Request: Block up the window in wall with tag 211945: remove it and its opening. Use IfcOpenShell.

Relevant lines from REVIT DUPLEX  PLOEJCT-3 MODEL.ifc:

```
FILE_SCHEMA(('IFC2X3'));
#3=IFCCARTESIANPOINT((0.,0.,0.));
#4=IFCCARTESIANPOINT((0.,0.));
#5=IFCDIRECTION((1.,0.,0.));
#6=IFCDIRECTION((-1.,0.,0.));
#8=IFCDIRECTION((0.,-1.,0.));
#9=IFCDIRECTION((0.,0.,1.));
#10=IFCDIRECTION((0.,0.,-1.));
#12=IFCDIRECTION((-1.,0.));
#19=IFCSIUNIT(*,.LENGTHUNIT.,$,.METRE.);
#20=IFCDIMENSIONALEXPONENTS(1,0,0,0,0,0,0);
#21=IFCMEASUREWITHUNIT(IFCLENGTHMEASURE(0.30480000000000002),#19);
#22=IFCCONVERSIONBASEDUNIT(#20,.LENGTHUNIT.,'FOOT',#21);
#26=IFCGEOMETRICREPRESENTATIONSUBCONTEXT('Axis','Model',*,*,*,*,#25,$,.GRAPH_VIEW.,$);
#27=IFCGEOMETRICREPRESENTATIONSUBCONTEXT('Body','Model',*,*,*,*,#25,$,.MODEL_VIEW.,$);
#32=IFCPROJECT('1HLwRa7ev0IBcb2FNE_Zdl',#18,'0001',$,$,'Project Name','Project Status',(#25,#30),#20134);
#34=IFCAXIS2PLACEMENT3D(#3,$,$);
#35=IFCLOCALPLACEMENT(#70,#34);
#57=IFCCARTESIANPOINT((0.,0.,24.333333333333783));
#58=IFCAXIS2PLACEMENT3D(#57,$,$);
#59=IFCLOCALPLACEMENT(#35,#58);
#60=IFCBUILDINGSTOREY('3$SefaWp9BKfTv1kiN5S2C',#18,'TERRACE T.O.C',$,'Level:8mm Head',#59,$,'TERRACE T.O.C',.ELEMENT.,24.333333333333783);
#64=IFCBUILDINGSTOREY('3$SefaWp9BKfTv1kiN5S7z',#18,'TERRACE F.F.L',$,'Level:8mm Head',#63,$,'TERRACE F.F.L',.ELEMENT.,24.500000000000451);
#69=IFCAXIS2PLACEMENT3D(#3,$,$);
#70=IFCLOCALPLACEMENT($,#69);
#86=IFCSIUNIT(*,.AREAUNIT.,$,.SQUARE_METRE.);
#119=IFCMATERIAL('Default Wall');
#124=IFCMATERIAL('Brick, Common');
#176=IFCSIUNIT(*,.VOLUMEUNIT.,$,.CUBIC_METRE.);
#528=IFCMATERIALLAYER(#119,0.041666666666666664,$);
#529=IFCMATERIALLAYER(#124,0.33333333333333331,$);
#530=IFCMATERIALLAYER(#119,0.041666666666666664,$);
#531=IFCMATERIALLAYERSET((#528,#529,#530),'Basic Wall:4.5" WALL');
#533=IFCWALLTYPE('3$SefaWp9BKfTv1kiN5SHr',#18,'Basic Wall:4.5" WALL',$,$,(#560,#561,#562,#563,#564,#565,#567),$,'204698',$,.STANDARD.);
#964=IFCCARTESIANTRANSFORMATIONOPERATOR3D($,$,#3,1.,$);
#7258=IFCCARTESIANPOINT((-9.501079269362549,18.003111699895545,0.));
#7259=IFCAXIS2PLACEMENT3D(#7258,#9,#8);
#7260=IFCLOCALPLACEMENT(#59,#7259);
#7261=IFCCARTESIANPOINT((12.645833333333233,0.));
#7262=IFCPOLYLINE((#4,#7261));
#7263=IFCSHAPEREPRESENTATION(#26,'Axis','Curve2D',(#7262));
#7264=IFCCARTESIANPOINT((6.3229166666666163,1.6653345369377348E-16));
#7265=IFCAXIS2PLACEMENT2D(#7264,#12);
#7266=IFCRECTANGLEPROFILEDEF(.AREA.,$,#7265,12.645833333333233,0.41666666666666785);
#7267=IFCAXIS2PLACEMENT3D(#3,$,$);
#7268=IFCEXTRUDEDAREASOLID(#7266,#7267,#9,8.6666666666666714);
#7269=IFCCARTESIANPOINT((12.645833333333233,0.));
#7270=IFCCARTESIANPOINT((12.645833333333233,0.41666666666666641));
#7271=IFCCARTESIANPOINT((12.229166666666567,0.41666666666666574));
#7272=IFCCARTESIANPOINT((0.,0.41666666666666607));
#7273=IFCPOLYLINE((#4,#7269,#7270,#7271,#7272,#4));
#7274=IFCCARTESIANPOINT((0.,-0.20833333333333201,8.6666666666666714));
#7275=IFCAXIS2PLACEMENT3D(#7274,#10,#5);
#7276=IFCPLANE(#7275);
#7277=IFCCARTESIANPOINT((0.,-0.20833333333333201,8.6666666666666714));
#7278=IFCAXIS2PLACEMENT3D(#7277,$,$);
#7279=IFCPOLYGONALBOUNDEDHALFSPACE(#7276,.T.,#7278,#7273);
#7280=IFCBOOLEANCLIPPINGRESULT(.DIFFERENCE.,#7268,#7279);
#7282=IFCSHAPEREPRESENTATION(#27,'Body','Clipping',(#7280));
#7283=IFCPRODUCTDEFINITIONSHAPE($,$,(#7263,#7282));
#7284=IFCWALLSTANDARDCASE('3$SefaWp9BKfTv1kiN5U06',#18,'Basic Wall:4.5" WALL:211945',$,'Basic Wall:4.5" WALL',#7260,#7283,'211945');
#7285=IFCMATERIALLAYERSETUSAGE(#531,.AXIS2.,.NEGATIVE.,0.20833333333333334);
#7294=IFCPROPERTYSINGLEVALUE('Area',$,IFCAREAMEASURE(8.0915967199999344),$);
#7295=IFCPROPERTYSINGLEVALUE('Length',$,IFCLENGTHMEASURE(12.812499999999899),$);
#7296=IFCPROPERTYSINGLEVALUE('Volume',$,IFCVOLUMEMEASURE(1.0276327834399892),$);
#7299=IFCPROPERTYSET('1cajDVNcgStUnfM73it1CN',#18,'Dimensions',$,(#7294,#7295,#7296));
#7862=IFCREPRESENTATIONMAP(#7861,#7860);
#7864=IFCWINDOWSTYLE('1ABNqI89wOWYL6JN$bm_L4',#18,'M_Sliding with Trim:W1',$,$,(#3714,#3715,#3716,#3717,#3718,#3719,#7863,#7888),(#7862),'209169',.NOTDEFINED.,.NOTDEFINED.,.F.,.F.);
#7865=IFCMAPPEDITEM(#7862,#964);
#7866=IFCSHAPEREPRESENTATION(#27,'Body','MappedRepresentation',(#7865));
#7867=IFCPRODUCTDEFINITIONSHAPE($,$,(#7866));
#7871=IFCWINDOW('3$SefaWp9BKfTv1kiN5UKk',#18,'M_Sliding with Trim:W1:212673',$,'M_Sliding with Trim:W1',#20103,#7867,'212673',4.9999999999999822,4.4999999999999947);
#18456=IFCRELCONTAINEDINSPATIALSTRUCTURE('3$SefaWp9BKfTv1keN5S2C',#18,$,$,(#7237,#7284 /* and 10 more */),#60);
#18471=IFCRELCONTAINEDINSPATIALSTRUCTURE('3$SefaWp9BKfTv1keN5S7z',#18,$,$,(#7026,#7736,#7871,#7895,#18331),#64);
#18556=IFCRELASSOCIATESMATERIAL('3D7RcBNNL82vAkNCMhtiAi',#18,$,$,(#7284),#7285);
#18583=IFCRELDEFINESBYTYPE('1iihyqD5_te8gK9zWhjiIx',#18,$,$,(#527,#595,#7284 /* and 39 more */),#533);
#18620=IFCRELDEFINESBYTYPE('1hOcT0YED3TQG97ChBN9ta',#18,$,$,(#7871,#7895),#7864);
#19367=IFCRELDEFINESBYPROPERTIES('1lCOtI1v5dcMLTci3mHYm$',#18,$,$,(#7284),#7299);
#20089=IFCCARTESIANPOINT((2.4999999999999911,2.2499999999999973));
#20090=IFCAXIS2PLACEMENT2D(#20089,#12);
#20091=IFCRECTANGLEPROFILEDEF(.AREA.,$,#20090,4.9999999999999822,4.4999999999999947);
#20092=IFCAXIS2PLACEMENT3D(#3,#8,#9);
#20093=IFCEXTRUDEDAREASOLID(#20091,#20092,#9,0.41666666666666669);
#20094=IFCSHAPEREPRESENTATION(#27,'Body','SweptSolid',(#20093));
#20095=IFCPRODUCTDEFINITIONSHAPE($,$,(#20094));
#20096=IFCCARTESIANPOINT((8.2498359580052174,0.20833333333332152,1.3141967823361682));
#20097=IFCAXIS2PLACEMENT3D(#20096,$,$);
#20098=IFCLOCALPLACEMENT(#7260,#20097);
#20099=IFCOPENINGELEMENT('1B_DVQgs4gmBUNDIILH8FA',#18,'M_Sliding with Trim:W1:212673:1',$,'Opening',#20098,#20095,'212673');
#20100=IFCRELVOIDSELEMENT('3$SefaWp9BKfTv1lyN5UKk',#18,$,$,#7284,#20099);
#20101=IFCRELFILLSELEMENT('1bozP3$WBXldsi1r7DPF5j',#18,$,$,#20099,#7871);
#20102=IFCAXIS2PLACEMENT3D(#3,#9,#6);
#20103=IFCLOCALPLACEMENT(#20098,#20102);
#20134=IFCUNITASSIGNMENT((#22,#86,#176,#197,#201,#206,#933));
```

```python
import ifcopenshell
import ifcopenshell.api.feature
import ifcopenshell.api.pset
import ifcopenshell.api.root
import ifcopenshell.geom
import ifcopenshell.util.element
import ifcopenshell.util.shape
import ifcopenshell.util.unit

model = ifcopenshell.open("REVIT DUPLEX  PLOEJCT-3 MODEL.ifc")
area_scale = ifcopenshell.util.unit.calculate_unit_scale(model, "AREAUNIT")
volume_scale = ifcopenshell.util.unit.calculate_unit_scale(model, "VOLUMEUNIT")
settings = ifcopenshell.geom.settings()


def volume(element):
    """Net volume in cubic metres, openings subtracted."""
    shape = ifcopenshell.geom.create_shape(settings, element)
    return ifcopenshell.util.shape.get_volume(shape.geometry)


window = model.by_id(7871)
opening = window.FillsVoids[0].RelatingOpeningElement
wall = opening.VoidsElements[0].RelatingBuildingElement
before = volume(wall)

ifcopenshell.api.root.remove_product(model, product=window)
ifcopenshell.api.feature.remove_feature(model, feature=opening)

after = volume(wall)
thickness = 0.127  # wall thickness in metres

# Update the wall's stored quantities.
pset = model.by_id(ifcopenshell.util.element.get_pset(wall, "Dimensions", should_inherit=False)["id"])
ifcopenshell.api.pset.edit_pset(model, pset=pset, properties={
    "Area": model.create_entity("IfcAreaMeasure", after / thickness / area_scale),
    "Volume": model.create_entity("IfcVolumeMeasure", after / volume_scale),
})

print(f"wall volume {before:.3f} -> {after:.3f} m3")

model.write("REVIT DUPLEX  PLOEJCT-3 MODEL_rev.ifc")
```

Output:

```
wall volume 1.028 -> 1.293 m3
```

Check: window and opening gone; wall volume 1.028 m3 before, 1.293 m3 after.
